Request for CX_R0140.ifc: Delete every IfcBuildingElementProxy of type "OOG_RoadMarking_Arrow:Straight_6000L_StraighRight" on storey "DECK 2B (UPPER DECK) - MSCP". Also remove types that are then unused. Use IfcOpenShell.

First a look at what the model holds.

```python
import ifcopenshell
import ifcopenshell.util.element

model = ifcopenshell.open("CX_R0140.ifc")
print(model.schema)
storey = next(s for s in model.by_type("IfcBuildingStorey") if s.Name == "DECK 2B (UPPER DECK) - MSCP")
proxies = [e for e in ifcopenshell.util.element.get_decomposition(storey) if e.is_a("IfcBuildingElementProxy")]
seen = {}
for e in proxies:
    element_type = ifcopenshell.util.element.get_type(e)
    name = element_type.Name if element_type not in (None, e) else None
    seen[name] = seen.get(name, 0) + 1
for name, count in sorted(seen.items(), key=str):
    print(count, "x", name)
```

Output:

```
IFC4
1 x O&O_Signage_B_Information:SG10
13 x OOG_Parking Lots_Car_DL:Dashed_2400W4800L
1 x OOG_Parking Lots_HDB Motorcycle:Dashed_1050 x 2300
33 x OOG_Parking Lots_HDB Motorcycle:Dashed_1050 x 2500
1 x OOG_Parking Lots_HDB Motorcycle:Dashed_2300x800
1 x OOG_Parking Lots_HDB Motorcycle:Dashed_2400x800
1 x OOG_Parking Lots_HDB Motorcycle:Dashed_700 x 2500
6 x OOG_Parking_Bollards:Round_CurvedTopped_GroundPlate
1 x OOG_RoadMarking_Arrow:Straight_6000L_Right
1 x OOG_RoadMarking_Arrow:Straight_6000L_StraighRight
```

```python
import ifcopenshell
import ifcopenshell.api.root
import ifcopenshell.util.element

model = ifcopenshell.open("CX_R0140.ifc")

storey = next(s for s in model.by_type("IfcBuildingStorey") if s.Name == "DECK 2B (UPPER DECK) - MSCP")
proxies = [e for e in ifcopenshell.util.element.get_decomposition(storey) if e.is_a("IfcBuildingElementProxy")]
targets = [e for e in proxies if (t := ifcopenshell.util.element.get_type(e)) not in (None, e) and t.Name == "OOG_RoadMarking_Arrow:Straight_6000L_StraighRight"]
types = {ifcopenshell.util.element.get_type(e) for e in targets} - {None, *targets}

for e in targets:
    ifcopenshell.api.root.remove_product(model, product=e)
print(len(targets), "removed")

unused = [t for t in types if not ifcopenshell.util.element.get_types(t)]
for t in unused:
    ifcopenshell.api.root.remove_product(model, product=t)
print(len(unused), "unused types removed")

model.write("CX_R0140_updated.ifc")
```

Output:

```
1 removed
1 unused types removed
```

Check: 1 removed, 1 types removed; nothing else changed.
